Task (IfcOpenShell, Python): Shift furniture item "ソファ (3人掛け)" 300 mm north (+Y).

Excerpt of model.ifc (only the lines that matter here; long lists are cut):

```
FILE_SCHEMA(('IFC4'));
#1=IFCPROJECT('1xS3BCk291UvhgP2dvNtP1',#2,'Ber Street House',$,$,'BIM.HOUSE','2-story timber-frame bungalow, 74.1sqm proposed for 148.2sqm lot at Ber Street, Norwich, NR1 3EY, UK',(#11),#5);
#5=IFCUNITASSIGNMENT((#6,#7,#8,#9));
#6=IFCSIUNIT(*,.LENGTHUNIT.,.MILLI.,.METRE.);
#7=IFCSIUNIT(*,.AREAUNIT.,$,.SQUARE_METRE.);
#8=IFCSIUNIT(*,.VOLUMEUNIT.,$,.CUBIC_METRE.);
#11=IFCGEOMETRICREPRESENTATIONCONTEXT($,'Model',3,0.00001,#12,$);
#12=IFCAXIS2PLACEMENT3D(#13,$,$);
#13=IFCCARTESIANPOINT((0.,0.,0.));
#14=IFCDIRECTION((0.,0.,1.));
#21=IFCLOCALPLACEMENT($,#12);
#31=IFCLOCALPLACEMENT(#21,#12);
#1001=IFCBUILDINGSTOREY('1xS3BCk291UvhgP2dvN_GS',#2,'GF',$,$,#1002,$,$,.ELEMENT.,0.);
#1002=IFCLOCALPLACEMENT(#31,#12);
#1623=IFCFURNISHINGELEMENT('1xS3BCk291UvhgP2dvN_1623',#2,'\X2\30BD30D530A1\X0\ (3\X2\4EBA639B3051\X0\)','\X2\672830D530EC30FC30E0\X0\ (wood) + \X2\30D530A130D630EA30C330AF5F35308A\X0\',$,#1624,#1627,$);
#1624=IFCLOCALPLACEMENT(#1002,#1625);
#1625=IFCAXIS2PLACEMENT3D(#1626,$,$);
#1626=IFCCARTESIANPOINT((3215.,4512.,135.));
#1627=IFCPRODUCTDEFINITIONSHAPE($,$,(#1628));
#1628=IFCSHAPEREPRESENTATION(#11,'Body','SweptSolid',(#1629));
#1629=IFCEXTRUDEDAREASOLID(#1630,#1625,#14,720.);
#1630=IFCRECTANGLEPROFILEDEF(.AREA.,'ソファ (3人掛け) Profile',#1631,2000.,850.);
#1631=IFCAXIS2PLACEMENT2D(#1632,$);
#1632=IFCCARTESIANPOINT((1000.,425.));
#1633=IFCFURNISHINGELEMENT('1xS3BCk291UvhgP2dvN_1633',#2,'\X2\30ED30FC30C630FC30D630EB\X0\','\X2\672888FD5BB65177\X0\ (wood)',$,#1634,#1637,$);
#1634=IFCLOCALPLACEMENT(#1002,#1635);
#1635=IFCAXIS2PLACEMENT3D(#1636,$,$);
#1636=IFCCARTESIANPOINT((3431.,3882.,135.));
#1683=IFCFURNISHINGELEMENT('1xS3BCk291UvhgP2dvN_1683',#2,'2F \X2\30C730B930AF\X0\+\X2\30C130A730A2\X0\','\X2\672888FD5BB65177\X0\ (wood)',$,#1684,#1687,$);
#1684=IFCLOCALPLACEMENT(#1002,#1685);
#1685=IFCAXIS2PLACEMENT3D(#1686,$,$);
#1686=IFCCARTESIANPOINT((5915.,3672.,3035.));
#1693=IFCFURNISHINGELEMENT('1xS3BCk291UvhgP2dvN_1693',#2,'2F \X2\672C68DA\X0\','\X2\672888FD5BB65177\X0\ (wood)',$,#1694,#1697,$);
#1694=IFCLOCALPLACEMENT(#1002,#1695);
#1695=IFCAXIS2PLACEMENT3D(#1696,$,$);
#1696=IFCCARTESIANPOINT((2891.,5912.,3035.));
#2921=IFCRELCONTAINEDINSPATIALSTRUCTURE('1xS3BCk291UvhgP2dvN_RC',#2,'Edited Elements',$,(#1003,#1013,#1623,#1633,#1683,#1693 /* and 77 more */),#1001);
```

```python
import ifcopenshell
import ifcopenshell.api.geometry
import ifcopenshell.util.placement

model = ifcopenshell.open("model.ifc")

item = model.by_guid("1xS3BCk291UvhgP2dvN_1623")
matrix = ifcopenshell.util.placement.get_local_placement(item.ObjectPlacement)
matrix[1, 3] += 300.0
ifcopenshell.api.geometry.edit_object_placement(model, product=item, matrix=matrix, is_si=False)

print(ifcopenshell.util.placement.get_local_placement(item.ObjectPlacement).round(3) + 0.0)

model.write("model_edited.ifc")
```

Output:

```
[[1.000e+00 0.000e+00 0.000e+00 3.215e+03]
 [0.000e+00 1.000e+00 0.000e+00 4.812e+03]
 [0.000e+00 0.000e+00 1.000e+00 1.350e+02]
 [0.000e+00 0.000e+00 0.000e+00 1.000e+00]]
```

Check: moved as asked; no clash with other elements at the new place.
